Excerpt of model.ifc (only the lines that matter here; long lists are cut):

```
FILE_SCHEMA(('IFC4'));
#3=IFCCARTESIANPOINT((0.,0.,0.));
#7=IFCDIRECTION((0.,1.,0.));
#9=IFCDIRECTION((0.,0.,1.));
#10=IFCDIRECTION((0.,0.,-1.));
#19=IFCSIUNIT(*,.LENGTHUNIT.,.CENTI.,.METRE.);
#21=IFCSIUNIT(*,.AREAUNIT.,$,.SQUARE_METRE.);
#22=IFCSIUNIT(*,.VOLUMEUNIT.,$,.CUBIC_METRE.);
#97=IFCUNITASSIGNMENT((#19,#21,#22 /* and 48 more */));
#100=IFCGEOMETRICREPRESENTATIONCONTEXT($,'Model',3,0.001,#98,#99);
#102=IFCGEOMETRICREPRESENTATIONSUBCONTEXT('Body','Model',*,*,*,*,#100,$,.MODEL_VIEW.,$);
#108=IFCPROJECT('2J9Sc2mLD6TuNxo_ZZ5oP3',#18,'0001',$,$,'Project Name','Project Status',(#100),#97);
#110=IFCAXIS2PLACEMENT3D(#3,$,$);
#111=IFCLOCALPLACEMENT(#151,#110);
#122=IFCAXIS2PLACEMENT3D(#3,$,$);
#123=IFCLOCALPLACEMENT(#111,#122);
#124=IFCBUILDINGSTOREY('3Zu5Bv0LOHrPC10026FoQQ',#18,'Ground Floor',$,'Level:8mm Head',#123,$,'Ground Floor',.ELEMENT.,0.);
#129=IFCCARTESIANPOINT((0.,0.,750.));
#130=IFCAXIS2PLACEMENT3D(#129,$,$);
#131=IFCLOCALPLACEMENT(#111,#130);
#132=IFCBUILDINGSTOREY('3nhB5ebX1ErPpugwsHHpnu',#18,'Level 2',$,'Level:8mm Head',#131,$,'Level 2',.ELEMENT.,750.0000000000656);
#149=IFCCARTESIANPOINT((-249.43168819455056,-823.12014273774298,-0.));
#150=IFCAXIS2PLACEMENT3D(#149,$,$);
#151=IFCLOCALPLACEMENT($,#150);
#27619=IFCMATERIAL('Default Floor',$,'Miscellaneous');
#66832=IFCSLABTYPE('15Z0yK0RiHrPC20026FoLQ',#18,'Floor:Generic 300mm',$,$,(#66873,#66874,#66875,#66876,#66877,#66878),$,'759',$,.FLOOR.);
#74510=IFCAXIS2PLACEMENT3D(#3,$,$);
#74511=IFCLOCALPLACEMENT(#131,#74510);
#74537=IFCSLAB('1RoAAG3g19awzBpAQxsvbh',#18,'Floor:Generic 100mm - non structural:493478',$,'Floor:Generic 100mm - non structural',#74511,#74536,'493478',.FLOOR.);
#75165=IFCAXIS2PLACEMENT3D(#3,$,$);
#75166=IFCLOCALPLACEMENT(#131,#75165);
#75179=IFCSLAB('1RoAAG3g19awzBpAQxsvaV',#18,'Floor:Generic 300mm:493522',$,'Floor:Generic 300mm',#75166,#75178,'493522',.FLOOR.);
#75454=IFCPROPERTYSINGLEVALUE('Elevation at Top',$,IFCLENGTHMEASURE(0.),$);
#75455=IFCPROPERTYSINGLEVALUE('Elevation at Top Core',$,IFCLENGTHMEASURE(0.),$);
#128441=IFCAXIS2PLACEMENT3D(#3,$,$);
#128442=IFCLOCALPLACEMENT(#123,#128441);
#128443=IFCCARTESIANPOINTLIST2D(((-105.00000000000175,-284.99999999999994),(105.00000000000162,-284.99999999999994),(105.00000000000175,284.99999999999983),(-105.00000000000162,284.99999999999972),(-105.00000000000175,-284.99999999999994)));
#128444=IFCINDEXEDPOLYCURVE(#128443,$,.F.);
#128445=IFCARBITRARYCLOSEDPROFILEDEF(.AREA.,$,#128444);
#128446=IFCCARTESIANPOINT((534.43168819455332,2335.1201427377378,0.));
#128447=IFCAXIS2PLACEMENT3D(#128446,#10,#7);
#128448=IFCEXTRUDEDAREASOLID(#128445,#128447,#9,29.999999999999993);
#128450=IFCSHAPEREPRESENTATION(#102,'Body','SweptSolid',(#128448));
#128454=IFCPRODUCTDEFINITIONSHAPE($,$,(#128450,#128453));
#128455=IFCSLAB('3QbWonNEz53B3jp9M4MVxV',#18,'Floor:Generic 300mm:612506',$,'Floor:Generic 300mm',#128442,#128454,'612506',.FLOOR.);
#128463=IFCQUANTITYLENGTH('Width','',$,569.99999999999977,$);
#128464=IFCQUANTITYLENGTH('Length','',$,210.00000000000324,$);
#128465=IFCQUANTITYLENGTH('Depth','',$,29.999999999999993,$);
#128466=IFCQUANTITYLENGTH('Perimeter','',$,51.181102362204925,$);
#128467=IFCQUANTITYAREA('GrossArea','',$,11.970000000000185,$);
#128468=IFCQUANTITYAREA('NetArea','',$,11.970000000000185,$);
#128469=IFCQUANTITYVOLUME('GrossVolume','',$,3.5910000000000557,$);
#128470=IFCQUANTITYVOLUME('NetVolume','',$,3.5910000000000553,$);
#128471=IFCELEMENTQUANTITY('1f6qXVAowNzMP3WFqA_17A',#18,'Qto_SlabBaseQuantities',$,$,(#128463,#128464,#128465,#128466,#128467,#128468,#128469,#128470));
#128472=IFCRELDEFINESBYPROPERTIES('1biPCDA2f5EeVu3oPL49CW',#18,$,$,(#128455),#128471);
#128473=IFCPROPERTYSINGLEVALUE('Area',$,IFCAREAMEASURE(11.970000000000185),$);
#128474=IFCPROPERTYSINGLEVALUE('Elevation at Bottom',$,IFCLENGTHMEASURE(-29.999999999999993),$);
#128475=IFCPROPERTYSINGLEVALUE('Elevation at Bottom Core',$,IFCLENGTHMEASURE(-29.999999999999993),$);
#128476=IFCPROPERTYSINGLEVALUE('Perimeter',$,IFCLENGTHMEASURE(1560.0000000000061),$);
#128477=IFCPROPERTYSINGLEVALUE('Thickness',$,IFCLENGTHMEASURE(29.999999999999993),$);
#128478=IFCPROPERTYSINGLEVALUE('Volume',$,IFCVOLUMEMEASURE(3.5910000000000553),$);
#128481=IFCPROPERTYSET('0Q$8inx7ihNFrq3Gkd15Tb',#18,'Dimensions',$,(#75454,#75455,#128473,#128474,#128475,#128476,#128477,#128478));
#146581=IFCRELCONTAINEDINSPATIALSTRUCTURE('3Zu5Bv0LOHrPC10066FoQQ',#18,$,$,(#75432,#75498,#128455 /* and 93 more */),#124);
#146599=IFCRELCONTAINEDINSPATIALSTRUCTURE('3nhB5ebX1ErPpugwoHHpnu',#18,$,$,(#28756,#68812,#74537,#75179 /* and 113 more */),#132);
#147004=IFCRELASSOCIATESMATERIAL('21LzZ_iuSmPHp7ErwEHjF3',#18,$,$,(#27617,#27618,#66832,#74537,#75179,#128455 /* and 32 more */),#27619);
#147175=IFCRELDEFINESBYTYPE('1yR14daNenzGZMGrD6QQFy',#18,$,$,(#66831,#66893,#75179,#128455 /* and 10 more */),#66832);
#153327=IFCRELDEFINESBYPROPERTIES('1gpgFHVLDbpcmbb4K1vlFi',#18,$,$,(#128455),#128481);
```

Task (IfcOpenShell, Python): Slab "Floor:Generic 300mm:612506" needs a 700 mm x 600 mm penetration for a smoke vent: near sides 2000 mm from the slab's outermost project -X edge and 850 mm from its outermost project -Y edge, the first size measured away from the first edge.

```python
import numpy as np
import ifcopenshell
import ifcopenshell.api.feature
import ifcopenshell.api.geometry
import ifcopenshell.api.pset
import ifcopenshell.api.root
import ifcopenshell.geom
import ifcopenshell.util.element
import ifcopenshell.util.placement
import ifcopenshell.util.representation
import ifcopenshell.util.shape
import ifcopenshell.util.unit

model = ifcopenshell.open("model.ifc")
unit_scale = ifcopenshell.util.unit.calculate_unit_scale(model)
area_scale = ifcopenshell.util.unit.calculate_unit_scale(model, "AREAUNIT")
volume_scale = ifcopenshell.util.unit.calculate_unit_scale(model, "VOLUMEUNIT")
settings = ifcopenshell.geom.settings()


def volume(element):
    """Net volume in cubic metres, openings subtracted."""
    shape = ifcopenshell.geom.create_shape(settings, element)
    return ifcopenshell.util.shape.get_volume(shape.geometry)


slab = model.by_guid("3QbWonNEz53B3jp9M4MVxV")
before = volume(slab)

# Extent in the slab's own axes, in metres. The edges named are its -X and -Y sides.
slab_shape = ifcopenshell.geom.create_shape(settings, slab)
vertices = ifcopenshell.util.shape.get_vertices(slab_shape.geometry)
x_min, y_min, bottom = vertices.min(axis=0)
top = vertices[:, 2].max()

opening = ifcopenshell.api.root.create_entity(model, ifc_class="IfcOpeningElement", name="Smoke vent opening", predefined_type="OPENING")
context = ifcopenshell.util.representation.get_context(model, "Model", "Body", "MODEL_VIEW")
width, depth = 0.7, 0.6
outline = [(0.0, 0.0), (width, 0.0), (width, depth), (0.0, depth), (0.0, 0.0)]
# Overshoot both faces by 50 mm so the cut is clean.
shape = ifcopenshell.api.geometry.add_slab_representation(
    model, context=context, depth=top - bottom + 0.1, polyline=outline
)
ifcopenshell.api.geometry.assign_representation(model, product=opening, representation=shape)

matrix = ifcopenshell.util.placement.get_local_placement(slab.ObjectPlacement)
matrix[:, 3] = matrix @ np.append(np.array([x_min + 2, y_min + 0.85, bottom - 0.05]) / unit_scale, 1.0)
ifcopenshell.api.geometry.edit_object_placement(model, product=opening, matrix=matrix, is_si=False)
ifcopenshell.api.feature.add_feature(model, feature=opening, element=slab)

after = volume(slab)

# Update the slab's stored quantities.
qto = model.by_id(ifcopenshell.util.element.get_pset(slab, "Qto_SlabBaseQuantities", should_inherit=False)["id"])
ifcopenshell.api.pset.edit_qto(model, qto=qto, properties={
    "NetArea": after / (top - bottom) / area_scale,
    "NetVolume": after / volume_scale,
})
pset = model.by_id(ifcopenshell.util.element.get_pset(slab, "Dimensions", should_inherit=False)["id"])
ifcopenshell.api.pset.edit_pset(model, pset=pset, properties={
    "Area": model.create_entity("IfcAreaMeasure", after / (top - bottom) / area_scale),
    "Volume": model.create_entity("IfcVolumeMeasure", after / volume_scale),
})

print(f"slab volume {before:.3f} -> {after:.3f} m3")

model.write("model_edited.ifc")
```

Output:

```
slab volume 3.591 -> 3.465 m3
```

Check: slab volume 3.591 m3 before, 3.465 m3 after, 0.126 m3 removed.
